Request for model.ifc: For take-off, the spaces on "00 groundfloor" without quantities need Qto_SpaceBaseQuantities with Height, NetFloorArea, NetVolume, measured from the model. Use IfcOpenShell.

First a look at what the model holds.

```python
import ifcopenshell
import ifcopenshell.util.element
import ifcopenshell.util.unit

model = ifcopenshell.open("model.ifc")
print(model.schema)
for unit_type in ("LENGTHUNIT", "AREAUNIT", "VOLUMEUNIT"):
    print(unit_type, ifcopenshell.util.unit.calculate_unit_scale(model, unit_type))
storey = next(s for s in model.by_type("IfcBuildingStorey") if s.Name == "00 groundfloor")
spaces = [e for e in ifcopenshell.util.element.get_decomposition(storey) if e.is_a("IfcSpace")]
for e in sorted(spaces, key=lambda e: e.id()):
    print(e.id(), e.is_a(), e.Name, list(ifcopenshell.util.element.get_psets(e, qtos_only=True)), sep=" | ")
```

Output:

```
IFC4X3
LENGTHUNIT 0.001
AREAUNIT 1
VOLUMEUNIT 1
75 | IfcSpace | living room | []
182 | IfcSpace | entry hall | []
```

```python
import ifcopenshell
import ifcopenshell.api.pset
import ifcopenshell.geom
import ifcopenshell.util.element
import ifcopenshell.util.shape
import ifcopenshell.util.unit

model = ifcopenshell.open("model.ifc")
unit_scale = ifcopenshell.util.unit.calculate_unit_scale(model)
area_scale = ifcopenshell.util.unit.calculate_unit_scale(model, "AREAUNIT")
volume_scale = ifcopenshell.util.unit.calculate_unit_scale(model, "VOLUMEUNIT")
settings = ifcopenshell.geom.settings()

storey = next(s for s in model.by_type("IfcBuildingStorey") if s.Name == "00 groundfloor")
spaces = [e for e in ifcopenshell.util.element.get_decomposition(storey) if e.is_a("IfcSpace")]

for e in sorted(spaces, key=lambda e: e.id()):
    if ifcopenshell.util.element.get_psets(e, qtos_only=True, should_inherit=False):
        continue
    # Geometry comes back in metres, in the element's own axes.
    shape = ifcopenshell.geom.create_shape(settings, e)
    values = {
        "Height": ifcopenshell.util.shape.get_z(shape.geometry) / unit_scale,
        "NetFloorArea": ifcopenshell.util.shape.get_footprint_area(shape.geometry) / area_scale,
        "NetVolume": ifcopenshell.util.shape.get_volume(shape.geometry) / volume_scale,
    }
    qto = ifcopenshell.api.pset.add_qto(model, product=e, name="Qto_SpaceBaseQuantities")
    ifcopenshell.api.pset.edit_qto(model, qto=qto, properties=values)
    print(e.id(), {k: round(v, 3) for k, v in values.items()})

model.write("model_v2.ifc")
```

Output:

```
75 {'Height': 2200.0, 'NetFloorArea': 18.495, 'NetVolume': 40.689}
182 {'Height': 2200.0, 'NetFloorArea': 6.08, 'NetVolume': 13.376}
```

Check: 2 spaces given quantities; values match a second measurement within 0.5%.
